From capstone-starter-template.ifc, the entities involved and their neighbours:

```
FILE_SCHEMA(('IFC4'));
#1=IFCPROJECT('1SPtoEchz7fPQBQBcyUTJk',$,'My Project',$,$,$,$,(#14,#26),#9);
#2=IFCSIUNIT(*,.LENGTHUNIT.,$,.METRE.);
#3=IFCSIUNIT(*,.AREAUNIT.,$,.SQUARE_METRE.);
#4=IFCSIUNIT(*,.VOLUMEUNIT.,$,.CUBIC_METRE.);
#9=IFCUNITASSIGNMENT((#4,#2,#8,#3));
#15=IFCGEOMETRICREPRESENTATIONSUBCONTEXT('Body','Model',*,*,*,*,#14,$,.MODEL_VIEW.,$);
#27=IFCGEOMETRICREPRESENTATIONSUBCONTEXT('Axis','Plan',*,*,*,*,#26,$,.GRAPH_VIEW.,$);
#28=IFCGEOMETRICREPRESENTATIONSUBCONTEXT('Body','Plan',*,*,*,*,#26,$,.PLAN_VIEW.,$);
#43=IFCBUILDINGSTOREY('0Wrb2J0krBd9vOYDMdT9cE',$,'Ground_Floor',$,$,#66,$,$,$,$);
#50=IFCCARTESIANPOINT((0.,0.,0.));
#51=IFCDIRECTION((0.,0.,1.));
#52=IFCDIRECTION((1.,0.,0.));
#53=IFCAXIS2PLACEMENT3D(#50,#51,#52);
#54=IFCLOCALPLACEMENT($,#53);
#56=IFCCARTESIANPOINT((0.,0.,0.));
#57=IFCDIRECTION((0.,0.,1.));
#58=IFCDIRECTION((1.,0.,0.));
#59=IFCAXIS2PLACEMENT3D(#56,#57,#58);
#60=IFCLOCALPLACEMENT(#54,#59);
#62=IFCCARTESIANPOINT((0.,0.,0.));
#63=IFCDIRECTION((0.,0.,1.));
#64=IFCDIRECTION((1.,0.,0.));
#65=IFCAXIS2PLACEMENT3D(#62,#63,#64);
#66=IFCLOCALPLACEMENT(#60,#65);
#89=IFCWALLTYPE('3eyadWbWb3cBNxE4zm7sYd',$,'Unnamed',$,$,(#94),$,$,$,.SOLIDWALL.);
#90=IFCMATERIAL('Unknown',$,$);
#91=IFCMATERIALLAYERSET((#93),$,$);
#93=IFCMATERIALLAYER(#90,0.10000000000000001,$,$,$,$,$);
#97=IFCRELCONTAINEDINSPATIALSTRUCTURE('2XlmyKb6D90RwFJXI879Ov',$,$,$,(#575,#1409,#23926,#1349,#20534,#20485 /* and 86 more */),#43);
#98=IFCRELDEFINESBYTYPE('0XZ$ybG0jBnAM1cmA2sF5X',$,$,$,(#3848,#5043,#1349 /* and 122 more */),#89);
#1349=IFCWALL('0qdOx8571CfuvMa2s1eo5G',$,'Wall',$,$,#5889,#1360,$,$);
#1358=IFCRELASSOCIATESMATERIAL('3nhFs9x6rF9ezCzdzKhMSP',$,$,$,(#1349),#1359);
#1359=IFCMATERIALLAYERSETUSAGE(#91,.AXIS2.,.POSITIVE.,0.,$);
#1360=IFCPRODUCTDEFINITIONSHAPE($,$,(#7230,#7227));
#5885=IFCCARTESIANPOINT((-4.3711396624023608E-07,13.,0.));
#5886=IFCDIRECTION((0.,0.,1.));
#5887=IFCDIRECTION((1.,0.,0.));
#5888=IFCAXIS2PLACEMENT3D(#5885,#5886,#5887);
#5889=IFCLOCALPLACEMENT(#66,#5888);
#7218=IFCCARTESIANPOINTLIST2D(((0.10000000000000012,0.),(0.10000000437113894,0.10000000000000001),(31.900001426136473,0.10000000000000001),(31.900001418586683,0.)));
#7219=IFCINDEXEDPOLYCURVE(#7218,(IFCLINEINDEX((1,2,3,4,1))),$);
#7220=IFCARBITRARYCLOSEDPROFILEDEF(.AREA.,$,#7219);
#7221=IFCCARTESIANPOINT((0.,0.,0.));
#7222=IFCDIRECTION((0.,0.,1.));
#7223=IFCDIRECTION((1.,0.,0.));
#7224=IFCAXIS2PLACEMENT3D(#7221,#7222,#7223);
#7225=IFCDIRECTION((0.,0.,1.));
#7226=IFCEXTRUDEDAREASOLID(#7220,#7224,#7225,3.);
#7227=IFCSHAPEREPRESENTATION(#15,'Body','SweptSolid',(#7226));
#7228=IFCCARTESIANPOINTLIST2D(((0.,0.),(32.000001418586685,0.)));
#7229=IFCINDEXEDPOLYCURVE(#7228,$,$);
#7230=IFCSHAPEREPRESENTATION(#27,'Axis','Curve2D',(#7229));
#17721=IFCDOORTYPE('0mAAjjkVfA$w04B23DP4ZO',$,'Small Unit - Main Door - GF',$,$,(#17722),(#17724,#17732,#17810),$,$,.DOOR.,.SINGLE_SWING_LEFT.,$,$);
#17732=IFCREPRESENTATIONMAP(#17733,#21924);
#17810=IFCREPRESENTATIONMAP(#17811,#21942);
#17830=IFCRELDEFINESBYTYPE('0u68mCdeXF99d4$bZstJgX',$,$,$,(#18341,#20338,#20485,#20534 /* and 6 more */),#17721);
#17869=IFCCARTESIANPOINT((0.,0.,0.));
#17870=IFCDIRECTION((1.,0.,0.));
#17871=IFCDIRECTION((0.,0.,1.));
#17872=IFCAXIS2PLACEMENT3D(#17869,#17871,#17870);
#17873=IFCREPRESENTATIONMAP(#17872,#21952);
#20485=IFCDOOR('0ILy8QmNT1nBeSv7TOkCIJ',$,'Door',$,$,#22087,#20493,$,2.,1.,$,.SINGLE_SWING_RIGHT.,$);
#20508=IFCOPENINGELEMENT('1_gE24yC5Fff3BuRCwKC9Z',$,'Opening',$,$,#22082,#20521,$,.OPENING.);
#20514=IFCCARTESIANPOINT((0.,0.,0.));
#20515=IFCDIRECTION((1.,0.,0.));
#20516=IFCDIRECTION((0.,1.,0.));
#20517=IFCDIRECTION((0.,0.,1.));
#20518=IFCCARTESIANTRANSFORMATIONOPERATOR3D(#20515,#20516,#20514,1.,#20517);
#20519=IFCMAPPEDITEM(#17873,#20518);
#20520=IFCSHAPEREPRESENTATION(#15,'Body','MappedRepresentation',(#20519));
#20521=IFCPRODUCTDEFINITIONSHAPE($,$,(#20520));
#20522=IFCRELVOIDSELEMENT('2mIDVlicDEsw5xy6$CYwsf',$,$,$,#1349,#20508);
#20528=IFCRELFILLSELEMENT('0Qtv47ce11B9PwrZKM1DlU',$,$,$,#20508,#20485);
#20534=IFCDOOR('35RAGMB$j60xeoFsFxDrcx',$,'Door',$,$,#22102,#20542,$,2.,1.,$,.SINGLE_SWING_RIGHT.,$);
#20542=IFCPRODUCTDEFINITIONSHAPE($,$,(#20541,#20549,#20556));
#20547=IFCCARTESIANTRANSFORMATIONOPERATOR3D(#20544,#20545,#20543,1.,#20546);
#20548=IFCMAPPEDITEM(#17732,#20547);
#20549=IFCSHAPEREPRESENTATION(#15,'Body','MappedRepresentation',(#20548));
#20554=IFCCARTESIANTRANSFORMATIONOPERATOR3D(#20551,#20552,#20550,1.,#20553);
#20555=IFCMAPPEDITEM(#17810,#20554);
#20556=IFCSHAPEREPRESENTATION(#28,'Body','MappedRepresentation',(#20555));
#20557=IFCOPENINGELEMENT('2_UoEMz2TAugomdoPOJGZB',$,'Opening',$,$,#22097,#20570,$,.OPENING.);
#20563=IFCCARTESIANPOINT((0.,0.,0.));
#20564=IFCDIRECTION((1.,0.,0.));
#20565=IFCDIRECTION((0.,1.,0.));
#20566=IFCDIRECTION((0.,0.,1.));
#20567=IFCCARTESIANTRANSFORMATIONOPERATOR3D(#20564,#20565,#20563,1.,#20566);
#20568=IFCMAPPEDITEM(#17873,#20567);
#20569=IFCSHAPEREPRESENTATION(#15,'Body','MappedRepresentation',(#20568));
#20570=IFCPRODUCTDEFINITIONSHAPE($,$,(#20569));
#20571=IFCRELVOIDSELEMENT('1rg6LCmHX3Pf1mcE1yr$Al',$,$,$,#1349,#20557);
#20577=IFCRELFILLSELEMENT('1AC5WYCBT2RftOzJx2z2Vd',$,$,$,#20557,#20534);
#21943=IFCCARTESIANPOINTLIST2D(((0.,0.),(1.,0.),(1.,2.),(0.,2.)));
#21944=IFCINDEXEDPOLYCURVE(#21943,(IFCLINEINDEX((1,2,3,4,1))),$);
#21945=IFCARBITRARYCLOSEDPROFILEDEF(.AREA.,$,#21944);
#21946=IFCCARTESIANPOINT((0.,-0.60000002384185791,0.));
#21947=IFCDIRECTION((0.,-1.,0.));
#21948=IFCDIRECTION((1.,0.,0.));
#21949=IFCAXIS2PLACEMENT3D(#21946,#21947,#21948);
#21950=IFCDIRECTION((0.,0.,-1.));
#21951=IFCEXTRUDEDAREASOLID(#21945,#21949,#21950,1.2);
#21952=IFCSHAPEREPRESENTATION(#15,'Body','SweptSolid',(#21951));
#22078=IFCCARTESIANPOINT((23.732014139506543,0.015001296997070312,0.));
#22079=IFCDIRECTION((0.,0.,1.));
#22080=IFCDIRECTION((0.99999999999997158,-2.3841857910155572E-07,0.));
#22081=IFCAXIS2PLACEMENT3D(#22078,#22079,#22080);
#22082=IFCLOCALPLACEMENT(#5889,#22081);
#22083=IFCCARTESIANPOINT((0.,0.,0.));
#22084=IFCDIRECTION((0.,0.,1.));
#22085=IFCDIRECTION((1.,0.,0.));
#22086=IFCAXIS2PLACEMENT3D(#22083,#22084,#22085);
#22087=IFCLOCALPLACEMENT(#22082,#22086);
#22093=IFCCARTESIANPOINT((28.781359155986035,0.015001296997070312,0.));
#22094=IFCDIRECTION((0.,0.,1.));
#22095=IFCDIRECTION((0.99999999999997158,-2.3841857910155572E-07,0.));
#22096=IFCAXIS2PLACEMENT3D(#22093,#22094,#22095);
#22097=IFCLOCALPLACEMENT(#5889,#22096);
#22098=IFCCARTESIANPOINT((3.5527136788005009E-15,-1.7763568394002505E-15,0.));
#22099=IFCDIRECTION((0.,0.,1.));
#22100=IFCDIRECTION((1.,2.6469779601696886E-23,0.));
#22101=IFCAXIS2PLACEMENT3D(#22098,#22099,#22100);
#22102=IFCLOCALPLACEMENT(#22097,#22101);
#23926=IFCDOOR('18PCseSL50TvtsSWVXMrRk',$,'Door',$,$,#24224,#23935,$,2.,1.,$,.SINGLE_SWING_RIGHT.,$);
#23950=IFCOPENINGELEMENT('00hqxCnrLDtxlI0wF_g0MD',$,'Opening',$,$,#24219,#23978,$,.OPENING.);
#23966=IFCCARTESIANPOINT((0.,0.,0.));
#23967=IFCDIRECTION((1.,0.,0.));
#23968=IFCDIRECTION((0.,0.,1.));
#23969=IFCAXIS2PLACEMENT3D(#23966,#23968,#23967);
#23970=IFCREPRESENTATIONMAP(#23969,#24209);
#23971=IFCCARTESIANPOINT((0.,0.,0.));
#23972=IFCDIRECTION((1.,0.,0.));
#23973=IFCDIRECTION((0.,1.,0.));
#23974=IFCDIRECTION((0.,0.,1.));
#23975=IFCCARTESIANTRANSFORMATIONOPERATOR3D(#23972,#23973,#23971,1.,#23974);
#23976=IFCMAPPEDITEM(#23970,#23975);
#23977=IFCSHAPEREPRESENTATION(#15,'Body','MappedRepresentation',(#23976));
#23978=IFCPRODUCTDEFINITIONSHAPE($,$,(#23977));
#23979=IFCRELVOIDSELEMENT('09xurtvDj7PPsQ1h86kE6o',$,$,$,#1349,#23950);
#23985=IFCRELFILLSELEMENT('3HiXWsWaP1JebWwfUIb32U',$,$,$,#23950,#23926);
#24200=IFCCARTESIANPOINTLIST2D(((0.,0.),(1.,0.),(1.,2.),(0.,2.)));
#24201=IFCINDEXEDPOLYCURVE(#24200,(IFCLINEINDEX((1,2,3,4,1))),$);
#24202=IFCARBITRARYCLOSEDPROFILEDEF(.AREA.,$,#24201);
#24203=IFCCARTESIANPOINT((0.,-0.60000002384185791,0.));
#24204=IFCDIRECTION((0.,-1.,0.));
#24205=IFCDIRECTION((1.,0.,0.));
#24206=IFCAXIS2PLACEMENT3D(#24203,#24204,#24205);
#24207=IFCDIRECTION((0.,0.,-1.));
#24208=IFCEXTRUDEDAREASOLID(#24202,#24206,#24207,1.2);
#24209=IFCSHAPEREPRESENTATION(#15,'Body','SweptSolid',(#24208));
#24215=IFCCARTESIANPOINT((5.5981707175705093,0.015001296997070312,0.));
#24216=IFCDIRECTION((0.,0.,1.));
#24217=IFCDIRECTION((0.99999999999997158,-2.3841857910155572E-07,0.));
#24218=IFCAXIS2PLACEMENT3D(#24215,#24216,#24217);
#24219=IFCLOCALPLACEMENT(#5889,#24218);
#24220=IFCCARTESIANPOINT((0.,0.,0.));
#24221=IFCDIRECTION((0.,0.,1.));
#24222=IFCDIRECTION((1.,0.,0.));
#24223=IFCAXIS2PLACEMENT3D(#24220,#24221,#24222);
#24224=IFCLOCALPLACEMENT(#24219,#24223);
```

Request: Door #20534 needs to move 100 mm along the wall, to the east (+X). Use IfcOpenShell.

```python
import ifcopenshell
import ifcopenshell.api.geometry
import ifcopenshell.util.placement
import ifcopenshell.util.unit

model = ifcopenshell.open("capstone-starter-template.ifc")
unit_scale = ifcopenshell.util.unit.calculate_unit_scale(model)

door = model.by_guid("35RAGMB$j60xeoFsFxDrcx")
opening = door.FillsVoids[0].RelatingOpeningElement
wall = opening.VoidsElements[0].RelatingBuildingElement

wall_matrix = ifcopenshell.util.placement.get_local_placement(wall.ObjectPlacement)
shift = wall_matrix[:3, 0] * 0.1 / unit_scale
before = ifcopenshell.util.placement.get_local_placement(door.ObjectPlacement)[:3, 3].copy()

# The door is placed relative to its opening, so it follows when the opening moves.
matrix = ifcopenshell.util.placement.get_local_placement(opening.ObjectPlacement)
matrix[:3, 3] += shift
ifcopenshell.api.geometry.edit_object_placement(
    model, product=opening, matrix=matrix, is_si=False, should_transform_children=True
)

after = ifcopenshell.util.placement.get_local_placement(door.ObjectPlacement)[:3, 3]
print("door moved by", (after - before).round(3) + 0.0)

model.write("capstone-starter-template-out.ifc")
```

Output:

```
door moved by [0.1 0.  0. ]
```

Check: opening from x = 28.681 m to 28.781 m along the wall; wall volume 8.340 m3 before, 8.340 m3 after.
